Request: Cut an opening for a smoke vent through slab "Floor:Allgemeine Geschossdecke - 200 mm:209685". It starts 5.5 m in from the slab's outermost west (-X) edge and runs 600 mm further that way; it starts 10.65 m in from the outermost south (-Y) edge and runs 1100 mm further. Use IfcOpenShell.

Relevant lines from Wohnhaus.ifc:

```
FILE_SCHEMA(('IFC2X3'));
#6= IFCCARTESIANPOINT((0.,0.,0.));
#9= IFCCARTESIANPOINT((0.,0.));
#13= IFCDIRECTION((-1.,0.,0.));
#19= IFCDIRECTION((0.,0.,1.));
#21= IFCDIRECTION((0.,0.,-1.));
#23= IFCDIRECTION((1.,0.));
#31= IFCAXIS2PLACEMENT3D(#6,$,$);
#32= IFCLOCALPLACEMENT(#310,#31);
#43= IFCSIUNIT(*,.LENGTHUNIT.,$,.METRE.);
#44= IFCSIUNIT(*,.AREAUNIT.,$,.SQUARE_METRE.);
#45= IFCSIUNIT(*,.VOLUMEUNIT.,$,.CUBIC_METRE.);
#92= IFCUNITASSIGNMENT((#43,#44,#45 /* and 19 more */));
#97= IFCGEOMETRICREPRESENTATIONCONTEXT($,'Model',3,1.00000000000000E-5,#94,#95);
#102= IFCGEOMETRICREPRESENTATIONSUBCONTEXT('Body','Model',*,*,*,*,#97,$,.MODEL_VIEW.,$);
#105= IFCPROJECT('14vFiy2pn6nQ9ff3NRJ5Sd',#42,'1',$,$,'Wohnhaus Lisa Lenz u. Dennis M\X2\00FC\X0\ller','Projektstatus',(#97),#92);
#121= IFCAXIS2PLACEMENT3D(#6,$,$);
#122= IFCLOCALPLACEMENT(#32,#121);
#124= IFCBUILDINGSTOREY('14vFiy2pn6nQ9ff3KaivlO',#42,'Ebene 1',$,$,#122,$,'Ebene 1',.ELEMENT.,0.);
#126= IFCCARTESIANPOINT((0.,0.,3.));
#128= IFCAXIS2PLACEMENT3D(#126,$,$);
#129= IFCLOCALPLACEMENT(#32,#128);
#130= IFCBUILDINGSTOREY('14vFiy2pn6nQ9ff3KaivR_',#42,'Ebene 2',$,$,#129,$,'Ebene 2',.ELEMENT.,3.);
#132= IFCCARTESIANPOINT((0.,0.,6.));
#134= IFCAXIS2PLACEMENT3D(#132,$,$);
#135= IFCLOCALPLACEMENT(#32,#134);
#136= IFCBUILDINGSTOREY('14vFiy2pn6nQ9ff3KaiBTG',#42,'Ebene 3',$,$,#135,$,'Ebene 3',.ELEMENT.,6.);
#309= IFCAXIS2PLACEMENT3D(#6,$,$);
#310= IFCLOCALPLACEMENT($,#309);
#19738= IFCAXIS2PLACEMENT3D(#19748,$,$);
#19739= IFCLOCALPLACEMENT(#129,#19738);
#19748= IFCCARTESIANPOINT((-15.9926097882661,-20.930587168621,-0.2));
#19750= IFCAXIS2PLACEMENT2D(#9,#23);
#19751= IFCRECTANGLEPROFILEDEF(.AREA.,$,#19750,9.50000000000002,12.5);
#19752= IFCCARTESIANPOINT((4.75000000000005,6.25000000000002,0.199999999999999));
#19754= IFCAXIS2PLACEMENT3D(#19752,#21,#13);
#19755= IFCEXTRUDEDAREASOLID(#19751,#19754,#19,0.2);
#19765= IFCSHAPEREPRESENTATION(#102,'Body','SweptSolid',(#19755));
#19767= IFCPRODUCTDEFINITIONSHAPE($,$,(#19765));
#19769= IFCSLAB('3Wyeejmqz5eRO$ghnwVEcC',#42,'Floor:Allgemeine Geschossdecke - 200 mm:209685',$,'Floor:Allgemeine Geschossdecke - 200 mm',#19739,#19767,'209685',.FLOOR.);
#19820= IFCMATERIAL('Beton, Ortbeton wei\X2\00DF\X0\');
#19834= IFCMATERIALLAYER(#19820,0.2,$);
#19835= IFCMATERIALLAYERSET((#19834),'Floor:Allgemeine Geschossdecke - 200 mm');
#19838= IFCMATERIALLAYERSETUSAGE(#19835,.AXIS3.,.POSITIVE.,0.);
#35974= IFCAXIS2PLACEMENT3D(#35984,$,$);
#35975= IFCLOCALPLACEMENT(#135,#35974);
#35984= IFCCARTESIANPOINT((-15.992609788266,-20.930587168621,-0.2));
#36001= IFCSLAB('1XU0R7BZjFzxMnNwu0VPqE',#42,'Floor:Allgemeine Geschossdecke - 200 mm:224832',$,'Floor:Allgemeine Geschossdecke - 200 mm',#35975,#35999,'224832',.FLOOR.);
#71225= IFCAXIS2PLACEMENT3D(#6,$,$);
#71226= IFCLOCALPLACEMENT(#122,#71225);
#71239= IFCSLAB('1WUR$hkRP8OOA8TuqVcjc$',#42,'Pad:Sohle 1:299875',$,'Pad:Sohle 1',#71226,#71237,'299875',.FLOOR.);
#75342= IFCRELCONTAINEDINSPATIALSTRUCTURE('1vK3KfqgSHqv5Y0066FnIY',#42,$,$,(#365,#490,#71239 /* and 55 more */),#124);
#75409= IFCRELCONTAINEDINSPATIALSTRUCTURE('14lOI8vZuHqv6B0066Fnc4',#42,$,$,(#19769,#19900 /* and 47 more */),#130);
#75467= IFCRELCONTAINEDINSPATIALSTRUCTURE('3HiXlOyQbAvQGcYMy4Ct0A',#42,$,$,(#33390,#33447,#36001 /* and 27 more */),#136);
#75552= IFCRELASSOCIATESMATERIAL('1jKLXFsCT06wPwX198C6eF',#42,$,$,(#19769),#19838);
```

```python
import numpy as np
import ifcopenshell
import ifcopenshell.api.feature
import ifcopenshell.api.geometry
import ifcopenshell.api.root
import ifcopenshell.geom
import ifcopenshell.util.placement
import ifcopenshell.util.representation
import ifcopenshell.util.shape
import ifcopenshell.util.unit

model = ifcopenshell.open("Wohnhaus.ifc")
unit_scale = ifcopenshell.util.unit.calculate_unit_scale(model)
settings = ifcopenshell.geom.settings()


def volume(element):
    """Net volume in cubic metres, openings subtracted."""
    shape = ifcopenshell.geom.create_shape(settings, element)
    return ifcopenshell.util.shape.get_volume(shape.geometry)


slab = model.by_guid("3Wyeejmqz5eRO$ghnwVEcC")
before = volume(slab)

# Extent in the slab's own axes, in metres. The edges named are its -X and -Y sides.
slab_shape = ifcopenshell.geom.create_shape(settings, slab)
vertices = ifcopenshell.util.shape.get_vertices(slab_shape.geometry)
x_min, y_min, bottom = vertices.min(axis=0)
top = vertices[:, 2].max()

opening = ifcopenshell.api.root.create_entity(model, ifc_class="IfcOpeningElement", name="Smoke vent opening")
context = ifcopenshell.util.representation.get_context(model, "Model", "Body", "MODEL_VIEW")
width, depth = 0.6, 1.1
outline = [(0.0, 0.0), (width, 0.0), (width, depth), (0.0, depth), (0.0, 0.0)]
# Overshoot both faces by 50 mm so the cut is clean.
shape = ifcopenshell.api.geometry.add_slab_representation(
    model, context=context, depth=top - bottom + 0.1, polyline=outline
)
ifcopenshell.api.geometry.assign_representation(model, product=opening, representation=shape)

matrix = ifcopenshell.util.placement.get_local_placement(slab.ObjectPlacement)
matrix[:, 3] = matrix @ np.append(np.array([x_min + 5.5, y_min + 10.65, bottom - 0.05]) / unit_scale, 1.0)
ifcopenshell.api.geometry.edit_object_placement(model, product=opening, matrix=matrix, is_si=False)
ifcopenshell.api.feature.add_feature(model, feature=opening, element=slab)

after = volume(slab)

print(f"slab volume {before:.3f} -> {after:.3f} m3")

model.write("Wohnhaus_edited.ifc")
```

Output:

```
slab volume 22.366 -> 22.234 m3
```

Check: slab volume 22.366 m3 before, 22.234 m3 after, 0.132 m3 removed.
